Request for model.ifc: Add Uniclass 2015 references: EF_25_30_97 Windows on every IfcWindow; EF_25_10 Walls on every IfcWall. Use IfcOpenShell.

First a look at what the model holds.

```python
import ifcopenshell

model = ifcopenshell.open("model.ifc")
print(model.schema)
print("classifications:", [c.Name for c in model.by_type("IfcClassification")])
for ifc_class in ("IfcDoor", "IfcRoof", "IfcStair", "IfcWall", "IfcWindow"):
    print(ifc_class, len(model.by_type(ifc_class)))
```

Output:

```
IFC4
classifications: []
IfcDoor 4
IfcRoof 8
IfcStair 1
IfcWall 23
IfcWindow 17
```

```python
import ifcopenshell
import ifcopenshell.api.classification

model = ifcopenshell.open("model.ifc")

system = ifcopenshell.api.classification.add_classification(model, classification="Uniclass 2015")

codes = {
    "IfcWindow": ("EF_25_30_97", "Windows"),
    "IfcWall": ("EF_25_10", "Walls"),
}
for ifc_class, (code, name) in codes.items():
    products = model.by_type(ifc_class)
    ifcopenshell.api.classification.add_reference(
        model, products=products, classification=system, identification=code, name=name
    )
    print(code, len(products))

model.write("model_updated.ifc")
```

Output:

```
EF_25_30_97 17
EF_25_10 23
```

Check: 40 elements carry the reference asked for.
